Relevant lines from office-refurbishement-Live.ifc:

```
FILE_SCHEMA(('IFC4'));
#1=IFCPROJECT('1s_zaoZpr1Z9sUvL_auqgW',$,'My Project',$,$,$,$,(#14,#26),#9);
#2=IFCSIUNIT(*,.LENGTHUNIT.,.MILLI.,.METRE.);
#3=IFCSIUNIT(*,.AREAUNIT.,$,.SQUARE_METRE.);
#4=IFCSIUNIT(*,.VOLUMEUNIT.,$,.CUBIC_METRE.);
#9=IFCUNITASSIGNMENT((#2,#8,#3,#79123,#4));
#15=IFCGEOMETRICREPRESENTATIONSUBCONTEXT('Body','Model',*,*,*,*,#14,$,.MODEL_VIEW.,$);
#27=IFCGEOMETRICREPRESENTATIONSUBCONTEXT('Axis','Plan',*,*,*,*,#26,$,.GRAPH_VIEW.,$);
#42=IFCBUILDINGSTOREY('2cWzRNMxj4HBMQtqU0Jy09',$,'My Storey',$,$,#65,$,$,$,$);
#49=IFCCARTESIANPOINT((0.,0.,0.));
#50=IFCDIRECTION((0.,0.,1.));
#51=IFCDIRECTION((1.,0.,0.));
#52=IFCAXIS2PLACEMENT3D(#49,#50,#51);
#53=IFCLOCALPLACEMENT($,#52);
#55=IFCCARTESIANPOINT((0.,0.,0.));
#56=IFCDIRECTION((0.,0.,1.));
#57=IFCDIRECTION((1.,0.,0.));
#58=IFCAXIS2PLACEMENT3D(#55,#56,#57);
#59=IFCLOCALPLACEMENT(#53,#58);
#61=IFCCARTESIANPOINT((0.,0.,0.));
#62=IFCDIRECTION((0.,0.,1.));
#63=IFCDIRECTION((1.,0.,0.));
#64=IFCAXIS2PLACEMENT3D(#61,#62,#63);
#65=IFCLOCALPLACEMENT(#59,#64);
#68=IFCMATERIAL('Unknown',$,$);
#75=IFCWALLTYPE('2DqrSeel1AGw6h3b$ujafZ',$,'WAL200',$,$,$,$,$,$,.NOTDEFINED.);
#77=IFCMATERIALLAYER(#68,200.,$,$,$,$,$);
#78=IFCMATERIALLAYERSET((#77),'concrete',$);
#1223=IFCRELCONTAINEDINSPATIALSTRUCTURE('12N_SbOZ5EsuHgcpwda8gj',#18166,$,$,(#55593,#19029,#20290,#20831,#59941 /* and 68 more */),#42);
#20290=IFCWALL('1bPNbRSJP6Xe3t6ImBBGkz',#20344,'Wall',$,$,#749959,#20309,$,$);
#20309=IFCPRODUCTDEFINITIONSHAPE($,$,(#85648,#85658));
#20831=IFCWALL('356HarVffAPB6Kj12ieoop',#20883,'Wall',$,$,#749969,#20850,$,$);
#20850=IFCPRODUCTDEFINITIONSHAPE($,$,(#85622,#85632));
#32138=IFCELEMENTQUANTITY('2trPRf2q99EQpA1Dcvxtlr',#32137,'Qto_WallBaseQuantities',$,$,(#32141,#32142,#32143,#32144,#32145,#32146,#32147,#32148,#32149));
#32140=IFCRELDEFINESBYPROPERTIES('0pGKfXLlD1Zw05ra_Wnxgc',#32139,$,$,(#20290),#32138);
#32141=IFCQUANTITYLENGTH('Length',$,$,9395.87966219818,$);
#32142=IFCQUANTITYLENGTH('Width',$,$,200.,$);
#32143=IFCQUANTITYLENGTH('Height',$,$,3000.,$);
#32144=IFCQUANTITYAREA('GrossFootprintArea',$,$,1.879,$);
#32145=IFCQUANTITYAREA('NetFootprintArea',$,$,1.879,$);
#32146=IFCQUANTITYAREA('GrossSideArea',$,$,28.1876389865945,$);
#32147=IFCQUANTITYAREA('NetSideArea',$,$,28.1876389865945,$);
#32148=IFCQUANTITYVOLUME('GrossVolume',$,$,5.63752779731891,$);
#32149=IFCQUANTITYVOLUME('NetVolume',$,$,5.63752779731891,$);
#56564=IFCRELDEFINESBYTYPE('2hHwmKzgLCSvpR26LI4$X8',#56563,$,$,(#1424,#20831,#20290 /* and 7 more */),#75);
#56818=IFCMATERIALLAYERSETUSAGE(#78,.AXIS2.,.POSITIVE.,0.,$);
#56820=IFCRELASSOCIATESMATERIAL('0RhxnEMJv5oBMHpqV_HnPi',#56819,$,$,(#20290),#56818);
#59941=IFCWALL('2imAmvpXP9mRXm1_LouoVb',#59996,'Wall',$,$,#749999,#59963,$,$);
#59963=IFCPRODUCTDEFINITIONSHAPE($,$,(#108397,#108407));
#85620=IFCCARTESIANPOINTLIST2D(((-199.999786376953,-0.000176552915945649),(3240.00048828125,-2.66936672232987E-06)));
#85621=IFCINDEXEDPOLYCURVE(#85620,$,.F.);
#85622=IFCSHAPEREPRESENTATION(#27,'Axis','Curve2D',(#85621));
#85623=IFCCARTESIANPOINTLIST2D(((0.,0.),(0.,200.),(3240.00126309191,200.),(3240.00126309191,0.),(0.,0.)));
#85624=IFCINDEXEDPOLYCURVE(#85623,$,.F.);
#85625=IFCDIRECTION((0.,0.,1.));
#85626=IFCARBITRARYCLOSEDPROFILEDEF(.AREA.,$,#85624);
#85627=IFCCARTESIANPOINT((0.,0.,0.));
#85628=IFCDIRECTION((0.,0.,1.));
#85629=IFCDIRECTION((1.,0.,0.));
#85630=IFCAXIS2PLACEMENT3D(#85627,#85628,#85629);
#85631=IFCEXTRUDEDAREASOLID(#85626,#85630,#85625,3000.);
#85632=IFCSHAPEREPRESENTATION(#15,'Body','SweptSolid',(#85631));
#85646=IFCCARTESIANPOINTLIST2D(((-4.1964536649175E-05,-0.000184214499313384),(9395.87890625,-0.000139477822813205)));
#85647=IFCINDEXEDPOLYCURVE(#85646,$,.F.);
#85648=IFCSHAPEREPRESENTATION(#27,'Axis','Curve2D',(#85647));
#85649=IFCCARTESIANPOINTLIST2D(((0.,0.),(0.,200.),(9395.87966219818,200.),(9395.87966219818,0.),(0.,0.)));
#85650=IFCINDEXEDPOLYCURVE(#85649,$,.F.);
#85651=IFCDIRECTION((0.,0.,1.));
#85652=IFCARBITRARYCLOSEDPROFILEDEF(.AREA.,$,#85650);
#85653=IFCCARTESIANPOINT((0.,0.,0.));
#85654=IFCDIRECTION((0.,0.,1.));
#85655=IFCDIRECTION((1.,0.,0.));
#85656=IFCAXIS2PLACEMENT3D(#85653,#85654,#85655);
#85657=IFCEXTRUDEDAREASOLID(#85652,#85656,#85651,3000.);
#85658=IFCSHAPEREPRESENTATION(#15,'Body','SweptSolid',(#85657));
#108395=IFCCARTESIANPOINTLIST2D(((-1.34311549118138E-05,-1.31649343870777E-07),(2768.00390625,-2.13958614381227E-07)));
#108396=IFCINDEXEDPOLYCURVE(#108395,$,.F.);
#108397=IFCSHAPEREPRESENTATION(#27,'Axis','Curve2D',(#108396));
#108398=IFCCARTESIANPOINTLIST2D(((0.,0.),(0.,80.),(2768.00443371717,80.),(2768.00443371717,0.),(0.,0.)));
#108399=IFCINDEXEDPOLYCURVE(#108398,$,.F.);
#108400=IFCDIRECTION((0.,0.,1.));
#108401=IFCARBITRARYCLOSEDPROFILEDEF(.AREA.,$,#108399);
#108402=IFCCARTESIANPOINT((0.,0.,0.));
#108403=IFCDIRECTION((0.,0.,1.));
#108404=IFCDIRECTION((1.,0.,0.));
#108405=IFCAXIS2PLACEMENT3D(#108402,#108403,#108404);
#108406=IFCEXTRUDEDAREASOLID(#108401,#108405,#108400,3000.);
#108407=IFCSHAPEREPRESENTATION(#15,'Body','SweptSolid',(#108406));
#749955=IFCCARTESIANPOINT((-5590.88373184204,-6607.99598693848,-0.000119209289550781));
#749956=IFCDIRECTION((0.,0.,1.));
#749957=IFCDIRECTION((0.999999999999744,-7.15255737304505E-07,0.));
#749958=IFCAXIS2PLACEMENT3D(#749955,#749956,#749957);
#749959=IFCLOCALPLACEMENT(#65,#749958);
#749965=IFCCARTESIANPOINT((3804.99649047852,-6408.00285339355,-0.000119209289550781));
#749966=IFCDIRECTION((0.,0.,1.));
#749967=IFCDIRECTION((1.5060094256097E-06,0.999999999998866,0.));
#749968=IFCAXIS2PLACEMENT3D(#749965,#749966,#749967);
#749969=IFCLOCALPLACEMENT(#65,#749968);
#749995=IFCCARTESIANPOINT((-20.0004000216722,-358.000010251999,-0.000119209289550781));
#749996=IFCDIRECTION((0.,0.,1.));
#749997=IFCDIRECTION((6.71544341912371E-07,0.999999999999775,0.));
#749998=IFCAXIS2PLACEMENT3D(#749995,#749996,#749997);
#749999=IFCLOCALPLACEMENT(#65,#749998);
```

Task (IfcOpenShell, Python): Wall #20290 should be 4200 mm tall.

```python
import ifcopenshell
import ifcopenshell.api.pset
import ifcopenshell.geom
import ifcopenshell.util.element
import ifcopenshell.util.representation
import ifcopenshell.util.shape
import ifcopenshell.util.unit

model = ifcopenshell.open("office-refurbishement-Live.ifc")
unit_scale = ifcopenshell.util.unit.calculate_unit_scale(model)
area_scale = ifcopenshell.util.unit.calculate_unit_scale(model, "AREAUNIT")
volume_scale = ifcopenshell.util.unit.calculate_unit_scale(model, "VOLUMEUNIT")
settings = ifcopenshell.geom.settings()


def volume(element):
    """Net volume in cubic metres, openings subtracted."""
    shape = ifcopenshell.geom.create_shape(settings, element)
    return ifcopenshell.util.shape.get_volume(shape.geometry)


wall = model.by_guid("1bPNbRSJP6Xe3t6ImBBGkz")
before = volume(wall)

body = ifcopenshell.util.representation.get_representation(wall, "Model", "Body")
solid = body.Items[0]
old_height = solid.Depth
solid.Depth = 4200.0
after = volume(wall)
thickness = 0.2  # wall thickness in metres

# Update the stored height, areas and volumes.
qto = model.by_id(ifcopenshell.util.element.get_pset(wall, "Qto_WallBaseQuantities", should_inherit=False)["id"])
ifcopenshell.api.pset.edit_qto(model, qto=qto, properties={
    "Height": solid.Depth,
    "GrossSideArea": ifcopenshell.util.element.get_pset(wall, "Qto_WallBaseQuantities", "GrossSideArea") * solid.Depth / old_height,
    "NetSideArea": after / thickness / area_scale,
    "GrossVolume": ifcopenshell.util.element.get_pset(wall, "Qto_WallBaseQuantities", "GrossVolume") * solid.Depth / old_height,
    "NetVolume": after / volume_scale,
})

print(f"height {old_height:g} -> {solid.Depth:g}, volume {before:.3f} -> {after:.3f} m3")

model.write("office-refurbishement-Live-out.ifc")
```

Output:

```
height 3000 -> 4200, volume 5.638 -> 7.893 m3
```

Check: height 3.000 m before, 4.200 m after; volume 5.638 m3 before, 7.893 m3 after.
